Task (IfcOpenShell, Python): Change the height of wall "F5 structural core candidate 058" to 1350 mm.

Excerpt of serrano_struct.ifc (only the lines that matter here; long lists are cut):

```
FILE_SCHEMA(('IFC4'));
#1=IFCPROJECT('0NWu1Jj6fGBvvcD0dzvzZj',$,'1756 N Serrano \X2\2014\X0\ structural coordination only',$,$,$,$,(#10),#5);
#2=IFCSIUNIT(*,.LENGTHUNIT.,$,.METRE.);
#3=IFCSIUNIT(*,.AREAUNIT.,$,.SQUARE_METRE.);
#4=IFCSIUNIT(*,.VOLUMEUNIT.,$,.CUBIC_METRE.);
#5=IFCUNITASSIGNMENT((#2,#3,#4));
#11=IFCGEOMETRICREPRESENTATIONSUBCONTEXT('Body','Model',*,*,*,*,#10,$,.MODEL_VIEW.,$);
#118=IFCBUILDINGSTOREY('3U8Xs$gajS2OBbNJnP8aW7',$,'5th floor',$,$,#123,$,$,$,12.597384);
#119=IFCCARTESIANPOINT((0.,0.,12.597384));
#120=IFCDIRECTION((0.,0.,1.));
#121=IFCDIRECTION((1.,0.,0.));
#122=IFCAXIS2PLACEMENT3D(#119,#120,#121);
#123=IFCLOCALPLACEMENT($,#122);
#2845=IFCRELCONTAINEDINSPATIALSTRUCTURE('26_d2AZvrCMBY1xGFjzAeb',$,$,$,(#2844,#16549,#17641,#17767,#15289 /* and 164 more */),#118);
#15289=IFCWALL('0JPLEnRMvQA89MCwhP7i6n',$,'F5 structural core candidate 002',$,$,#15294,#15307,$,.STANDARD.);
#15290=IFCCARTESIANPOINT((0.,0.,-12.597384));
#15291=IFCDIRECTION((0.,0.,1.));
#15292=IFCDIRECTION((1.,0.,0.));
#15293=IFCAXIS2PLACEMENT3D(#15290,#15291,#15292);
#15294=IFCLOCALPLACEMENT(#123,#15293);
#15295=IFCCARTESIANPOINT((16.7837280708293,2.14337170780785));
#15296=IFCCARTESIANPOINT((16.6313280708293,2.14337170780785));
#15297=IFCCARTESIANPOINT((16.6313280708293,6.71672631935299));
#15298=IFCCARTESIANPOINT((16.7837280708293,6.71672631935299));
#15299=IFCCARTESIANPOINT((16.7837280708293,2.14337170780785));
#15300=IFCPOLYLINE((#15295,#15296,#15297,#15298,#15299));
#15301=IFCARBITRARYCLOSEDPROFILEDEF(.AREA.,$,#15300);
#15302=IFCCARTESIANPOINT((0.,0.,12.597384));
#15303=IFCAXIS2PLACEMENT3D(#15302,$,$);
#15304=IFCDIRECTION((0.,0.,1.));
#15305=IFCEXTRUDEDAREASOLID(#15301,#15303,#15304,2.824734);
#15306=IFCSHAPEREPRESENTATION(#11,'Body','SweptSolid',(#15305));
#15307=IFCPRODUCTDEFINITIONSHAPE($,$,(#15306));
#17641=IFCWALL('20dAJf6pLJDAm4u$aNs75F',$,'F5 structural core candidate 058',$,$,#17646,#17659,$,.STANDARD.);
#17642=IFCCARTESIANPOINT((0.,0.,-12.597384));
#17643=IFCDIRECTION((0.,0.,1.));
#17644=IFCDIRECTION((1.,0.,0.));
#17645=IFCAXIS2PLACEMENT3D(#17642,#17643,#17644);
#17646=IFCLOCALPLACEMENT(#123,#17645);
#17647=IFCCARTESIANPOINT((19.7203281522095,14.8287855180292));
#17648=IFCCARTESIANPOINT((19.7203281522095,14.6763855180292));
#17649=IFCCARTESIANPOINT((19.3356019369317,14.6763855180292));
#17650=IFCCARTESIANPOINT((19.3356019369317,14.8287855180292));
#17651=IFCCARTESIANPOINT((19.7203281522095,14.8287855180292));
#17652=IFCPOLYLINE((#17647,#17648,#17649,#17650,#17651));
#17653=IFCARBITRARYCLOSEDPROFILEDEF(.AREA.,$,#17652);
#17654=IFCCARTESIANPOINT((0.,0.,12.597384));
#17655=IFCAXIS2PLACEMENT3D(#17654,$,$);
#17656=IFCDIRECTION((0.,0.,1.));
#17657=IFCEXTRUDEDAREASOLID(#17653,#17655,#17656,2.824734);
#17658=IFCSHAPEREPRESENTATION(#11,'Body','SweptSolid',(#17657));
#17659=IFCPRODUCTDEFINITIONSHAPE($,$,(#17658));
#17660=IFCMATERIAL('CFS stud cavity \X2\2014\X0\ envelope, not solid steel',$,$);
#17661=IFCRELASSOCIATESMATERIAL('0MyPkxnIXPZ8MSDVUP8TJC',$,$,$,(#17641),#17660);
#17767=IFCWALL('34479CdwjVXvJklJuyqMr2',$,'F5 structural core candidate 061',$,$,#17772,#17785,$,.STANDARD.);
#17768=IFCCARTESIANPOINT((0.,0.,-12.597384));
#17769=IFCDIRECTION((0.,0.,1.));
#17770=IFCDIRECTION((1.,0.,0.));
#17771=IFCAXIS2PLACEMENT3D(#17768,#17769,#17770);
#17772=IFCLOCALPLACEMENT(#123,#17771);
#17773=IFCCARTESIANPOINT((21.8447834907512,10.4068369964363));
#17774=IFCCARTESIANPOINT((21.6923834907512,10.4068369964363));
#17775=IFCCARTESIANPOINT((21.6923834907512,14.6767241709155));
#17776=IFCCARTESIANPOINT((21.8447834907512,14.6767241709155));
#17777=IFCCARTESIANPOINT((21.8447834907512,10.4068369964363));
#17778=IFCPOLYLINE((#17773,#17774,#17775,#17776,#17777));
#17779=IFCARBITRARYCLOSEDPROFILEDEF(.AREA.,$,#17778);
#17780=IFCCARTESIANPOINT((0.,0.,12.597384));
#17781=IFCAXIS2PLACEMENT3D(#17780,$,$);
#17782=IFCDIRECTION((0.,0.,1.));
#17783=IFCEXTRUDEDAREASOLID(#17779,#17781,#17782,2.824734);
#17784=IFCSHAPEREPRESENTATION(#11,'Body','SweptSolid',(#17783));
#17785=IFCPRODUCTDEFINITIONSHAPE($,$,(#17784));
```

```python
import ifcopenshell
import ifcopenshell.geom
import ifcopenshell.util.representation
import ifcopenshell.util.shape
import ifcopenshell.util.unit

model = ifcopenshell.open("serrano_struct.ifc")
unit_scale = ifcopenshell.util.unit.calculate_unit_scale(model)
settings = ifcopenshell.geom.settings()


def volume(element):
    """Net volume in cubic metres, openings subtracted."""
    shape = ifcopenshell.geom.create_shape(settings, element)
    return ifcopenshell.util.shape.get_volume(shape.geometry)


wall = model.by_id(17641)
before = volume(wall)

body = ifcopenshell.util.representation.get_representation(wall, "Model", "Body")
solid = body.Items[0]
old_height = solid.Depth
solid.Depth = 1.35 / unit_scale
after = volume(wall)

print(f"height {old_height:g} -> {solid.Depth:g}, volume {before:.3f} -> {after:.3f} m3")

model.write("serrano_struct_edited.ifc")
```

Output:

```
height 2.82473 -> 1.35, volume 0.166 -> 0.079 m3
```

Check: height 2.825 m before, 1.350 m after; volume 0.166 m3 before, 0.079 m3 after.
